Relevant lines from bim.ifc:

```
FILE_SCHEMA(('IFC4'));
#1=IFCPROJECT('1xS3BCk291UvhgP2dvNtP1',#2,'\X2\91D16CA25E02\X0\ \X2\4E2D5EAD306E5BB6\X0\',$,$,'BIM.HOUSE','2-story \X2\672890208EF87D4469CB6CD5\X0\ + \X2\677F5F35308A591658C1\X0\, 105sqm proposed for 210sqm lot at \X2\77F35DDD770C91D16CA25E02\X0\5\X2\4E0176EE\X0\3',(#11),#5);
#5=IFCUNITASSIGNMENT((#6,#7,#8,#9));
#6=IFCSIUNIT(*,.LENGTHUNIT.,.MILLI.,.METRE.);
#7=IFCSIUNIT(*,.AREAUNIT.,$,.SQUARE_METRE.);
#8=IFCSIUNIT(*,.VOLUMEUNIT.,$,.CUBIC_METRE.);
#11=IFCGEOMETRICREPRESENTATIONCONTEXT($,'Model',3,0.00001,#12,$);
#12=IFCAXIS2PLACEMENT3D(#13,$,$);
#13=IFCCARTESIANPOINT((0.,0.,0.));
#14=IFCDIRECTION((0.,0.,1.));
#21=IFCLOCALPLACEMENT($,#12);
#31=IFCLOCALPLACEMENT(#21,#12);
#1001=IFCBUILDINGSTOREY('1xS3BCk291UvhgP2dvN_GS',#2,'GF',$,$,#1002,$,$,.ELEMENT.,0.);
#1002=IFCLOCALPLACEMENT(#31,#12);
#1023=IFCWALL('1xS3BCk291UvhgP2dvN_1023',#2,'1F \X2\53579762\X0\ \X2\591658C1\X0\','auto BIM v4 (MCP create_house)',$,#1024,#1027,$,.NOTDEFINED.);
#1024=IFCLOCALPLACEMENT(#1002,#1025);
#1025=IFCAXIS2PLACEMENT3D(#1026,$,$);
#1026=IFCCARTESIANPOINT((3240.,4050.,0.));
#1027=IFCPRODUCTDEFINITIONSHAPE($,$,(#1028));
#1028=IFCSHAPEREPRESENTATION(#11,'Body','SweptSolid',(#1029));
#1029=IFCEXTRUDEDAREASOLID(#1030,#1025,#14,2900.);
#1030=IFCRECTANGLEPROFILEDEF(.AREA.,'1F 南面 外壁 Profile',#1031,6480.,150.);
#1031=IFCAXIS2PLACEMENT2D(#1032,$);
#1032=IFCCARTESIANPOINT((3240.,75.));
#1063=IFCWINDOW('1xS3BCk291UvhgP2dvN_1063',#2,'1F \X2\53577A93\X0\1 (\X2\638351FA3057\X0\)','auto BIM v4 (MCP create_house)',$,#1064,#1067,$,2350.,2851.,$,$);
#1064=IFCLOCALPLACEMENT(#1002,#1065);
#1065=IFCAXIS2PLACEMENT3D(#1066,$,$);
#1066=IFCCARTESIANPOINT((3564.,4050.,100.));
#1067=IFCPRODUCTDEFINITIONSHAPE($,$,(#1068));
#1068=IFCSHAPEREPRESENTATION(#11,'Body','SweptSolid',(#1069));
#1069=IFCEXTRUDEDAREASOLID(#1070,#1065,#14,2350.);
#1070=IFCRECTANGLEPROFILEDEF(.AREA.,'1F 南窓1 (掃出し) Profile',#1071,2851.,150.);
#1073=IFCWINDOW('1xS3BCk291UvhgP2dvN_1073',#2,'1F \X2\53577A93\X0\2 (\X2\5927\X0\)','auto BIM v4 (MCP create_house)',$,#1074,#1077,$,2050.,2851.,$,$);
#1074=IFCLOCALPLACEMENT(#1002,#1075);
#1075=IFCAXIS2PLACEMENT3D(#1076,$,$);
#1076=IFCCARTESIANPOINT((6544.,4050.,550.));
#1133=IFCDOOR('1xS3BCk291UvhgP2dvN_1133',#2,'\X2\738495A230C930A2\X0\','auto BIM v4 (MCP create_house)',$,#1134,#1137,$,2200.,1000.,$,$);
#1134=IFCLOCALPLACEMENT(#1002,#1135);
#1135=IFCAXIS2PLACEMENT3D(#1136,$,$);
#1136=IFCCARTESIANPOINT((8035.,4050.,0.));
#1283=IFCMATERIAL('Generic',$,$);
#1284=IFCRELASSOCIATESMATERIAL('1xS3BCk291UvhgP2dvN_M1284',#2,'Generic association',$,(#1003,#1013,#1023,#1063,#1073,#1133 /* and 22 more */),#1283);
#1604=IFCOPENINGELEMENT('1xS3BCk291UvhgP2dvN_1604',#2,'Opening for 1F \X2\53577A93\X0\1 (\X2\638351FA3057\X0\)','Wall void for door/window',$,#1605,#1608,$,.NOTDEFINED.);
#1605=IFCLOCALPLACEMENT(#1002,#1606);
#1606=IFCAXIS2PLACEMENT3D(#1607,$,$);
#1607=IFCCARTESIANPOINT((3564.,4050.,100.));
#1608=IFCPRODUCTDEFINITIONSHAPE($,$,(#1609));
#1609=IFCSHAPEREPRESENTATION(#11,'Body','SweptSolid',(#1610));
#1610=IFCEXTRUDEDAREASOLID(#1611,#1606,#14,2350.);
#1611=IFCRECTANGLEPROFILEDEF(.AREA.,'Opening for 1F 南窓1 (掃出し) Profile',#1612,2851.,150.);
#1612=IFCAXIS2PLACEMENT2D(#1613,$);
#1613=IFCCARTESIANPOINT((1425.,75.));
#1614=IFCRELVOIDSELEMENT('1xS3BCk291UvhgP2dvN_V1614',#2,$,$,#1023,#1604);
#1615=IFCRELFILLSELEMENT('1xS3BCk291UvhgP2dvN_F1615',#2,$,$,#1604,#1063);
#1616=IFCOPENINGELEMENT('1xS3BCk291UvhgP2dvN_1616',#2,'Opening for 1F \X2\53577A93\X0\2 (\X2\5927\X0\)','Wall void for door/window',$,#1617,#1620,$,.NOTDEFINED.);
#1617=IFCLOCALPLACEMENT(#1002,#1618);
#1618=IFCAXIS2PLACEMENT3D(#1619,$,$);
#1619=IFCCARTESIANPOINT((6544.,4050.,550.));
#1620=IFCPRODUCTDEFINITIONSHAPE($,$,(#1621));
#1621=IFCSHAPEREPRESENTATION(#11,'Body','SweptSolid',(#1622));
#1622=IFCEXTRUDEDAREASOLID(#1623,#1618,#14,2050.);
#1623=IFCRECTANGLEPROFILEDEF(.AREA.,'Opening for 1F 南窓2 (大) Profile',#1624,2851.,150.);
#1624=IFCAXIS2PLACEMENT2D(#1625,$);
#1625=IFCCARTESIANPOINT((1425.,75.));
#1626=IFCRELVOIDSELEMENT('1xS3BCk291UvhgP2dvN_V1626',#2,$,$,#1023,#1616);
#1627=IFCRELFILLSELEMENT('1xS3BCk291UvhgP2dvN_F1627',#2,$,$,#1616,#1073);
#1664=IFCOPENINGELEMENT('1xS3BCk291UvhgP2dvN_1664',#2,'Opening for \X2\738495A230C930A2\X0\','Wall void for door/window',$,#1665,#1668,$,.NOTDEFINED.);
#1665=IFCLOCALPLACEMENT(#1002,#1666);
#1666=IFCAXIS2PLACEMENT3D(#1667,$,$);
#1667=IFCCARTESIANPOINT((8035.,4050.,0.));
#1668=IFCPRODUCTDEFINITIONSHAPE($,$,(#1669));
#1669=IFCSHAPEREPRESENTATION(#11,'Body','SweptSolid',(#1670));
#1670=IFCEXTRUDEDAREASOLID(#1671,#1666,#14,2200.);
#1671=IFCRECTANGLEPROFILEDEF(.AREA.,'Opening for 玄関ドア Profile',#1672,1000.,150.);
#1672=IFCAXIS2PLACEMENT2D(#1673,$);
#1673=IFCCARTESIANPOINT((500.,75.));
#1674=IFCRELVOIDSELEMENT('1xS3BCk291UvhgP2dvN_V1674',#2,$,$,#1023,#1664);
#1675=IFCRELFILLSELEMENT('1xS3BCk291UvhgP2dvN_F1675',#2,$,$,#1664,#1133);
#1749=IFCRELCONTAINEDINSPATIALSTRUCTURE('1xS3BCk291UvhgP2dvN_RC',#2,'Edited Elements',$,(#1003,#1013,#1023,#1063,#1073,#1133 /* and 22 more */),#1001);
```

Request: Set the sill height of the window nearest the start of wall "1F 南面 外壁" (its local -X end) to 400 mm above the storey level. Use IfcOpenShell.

```python
import numpy as np
import ifcopenshell
import ifcopenshell.api.geometry
import ifcopenshell.geom
import ifcopenshell.util.element
import ifcopenshell.util.placement
import ifcopenshell.util.shape
import ifcopenshell.util.unit

model = ifcopenshell.open("bim.ifc")
unit_scale = ifcopenshell.util.unit.calculate_unit_scale(model)

window = model.by_guid("1xS3BCk291UvhgP2dvN_1063")
opening = window.FillsVoids[0].RelatingOpeningElement
storey = ifcopenshell.util.element.get_container(window, ifc_class="IfcBuildingStorey")
level = ifcopenshell.util.placement.get_local_placement(storey.ObjectPlacement)[2, 3]

# The opening's origin need not be at the sill, so measure its lowest point.
shape = ifcopenshell.geom.create_shape(ifcopenshell.geom.settings(), opening)
bottom = ifcopenshell.util.shape.get_shape_bottom_elevation(shape, shape.geometry) / unit_scale
dz = level + 400.0 - bottom

shift = np.array([0.0, 0.0, dz])
# The window is not placed relative to its opening, so move both.
for product in (opening, window):
    matrix = ifcopenshell.util.placement.get_local_placement(product.ObjectPlacement)
    matrix[:3, 3] += shift
    ifcopenshell.api.geometry.edit_object_placement(model, product=product, matrix=matrix, is_si=False)

print(f"moved by {dz * unit_scale:+.3f} m")

model.write("bim_updated.ifc")
```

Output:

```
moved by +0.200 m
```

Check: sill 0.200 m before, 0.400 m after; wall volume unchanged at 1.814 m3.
